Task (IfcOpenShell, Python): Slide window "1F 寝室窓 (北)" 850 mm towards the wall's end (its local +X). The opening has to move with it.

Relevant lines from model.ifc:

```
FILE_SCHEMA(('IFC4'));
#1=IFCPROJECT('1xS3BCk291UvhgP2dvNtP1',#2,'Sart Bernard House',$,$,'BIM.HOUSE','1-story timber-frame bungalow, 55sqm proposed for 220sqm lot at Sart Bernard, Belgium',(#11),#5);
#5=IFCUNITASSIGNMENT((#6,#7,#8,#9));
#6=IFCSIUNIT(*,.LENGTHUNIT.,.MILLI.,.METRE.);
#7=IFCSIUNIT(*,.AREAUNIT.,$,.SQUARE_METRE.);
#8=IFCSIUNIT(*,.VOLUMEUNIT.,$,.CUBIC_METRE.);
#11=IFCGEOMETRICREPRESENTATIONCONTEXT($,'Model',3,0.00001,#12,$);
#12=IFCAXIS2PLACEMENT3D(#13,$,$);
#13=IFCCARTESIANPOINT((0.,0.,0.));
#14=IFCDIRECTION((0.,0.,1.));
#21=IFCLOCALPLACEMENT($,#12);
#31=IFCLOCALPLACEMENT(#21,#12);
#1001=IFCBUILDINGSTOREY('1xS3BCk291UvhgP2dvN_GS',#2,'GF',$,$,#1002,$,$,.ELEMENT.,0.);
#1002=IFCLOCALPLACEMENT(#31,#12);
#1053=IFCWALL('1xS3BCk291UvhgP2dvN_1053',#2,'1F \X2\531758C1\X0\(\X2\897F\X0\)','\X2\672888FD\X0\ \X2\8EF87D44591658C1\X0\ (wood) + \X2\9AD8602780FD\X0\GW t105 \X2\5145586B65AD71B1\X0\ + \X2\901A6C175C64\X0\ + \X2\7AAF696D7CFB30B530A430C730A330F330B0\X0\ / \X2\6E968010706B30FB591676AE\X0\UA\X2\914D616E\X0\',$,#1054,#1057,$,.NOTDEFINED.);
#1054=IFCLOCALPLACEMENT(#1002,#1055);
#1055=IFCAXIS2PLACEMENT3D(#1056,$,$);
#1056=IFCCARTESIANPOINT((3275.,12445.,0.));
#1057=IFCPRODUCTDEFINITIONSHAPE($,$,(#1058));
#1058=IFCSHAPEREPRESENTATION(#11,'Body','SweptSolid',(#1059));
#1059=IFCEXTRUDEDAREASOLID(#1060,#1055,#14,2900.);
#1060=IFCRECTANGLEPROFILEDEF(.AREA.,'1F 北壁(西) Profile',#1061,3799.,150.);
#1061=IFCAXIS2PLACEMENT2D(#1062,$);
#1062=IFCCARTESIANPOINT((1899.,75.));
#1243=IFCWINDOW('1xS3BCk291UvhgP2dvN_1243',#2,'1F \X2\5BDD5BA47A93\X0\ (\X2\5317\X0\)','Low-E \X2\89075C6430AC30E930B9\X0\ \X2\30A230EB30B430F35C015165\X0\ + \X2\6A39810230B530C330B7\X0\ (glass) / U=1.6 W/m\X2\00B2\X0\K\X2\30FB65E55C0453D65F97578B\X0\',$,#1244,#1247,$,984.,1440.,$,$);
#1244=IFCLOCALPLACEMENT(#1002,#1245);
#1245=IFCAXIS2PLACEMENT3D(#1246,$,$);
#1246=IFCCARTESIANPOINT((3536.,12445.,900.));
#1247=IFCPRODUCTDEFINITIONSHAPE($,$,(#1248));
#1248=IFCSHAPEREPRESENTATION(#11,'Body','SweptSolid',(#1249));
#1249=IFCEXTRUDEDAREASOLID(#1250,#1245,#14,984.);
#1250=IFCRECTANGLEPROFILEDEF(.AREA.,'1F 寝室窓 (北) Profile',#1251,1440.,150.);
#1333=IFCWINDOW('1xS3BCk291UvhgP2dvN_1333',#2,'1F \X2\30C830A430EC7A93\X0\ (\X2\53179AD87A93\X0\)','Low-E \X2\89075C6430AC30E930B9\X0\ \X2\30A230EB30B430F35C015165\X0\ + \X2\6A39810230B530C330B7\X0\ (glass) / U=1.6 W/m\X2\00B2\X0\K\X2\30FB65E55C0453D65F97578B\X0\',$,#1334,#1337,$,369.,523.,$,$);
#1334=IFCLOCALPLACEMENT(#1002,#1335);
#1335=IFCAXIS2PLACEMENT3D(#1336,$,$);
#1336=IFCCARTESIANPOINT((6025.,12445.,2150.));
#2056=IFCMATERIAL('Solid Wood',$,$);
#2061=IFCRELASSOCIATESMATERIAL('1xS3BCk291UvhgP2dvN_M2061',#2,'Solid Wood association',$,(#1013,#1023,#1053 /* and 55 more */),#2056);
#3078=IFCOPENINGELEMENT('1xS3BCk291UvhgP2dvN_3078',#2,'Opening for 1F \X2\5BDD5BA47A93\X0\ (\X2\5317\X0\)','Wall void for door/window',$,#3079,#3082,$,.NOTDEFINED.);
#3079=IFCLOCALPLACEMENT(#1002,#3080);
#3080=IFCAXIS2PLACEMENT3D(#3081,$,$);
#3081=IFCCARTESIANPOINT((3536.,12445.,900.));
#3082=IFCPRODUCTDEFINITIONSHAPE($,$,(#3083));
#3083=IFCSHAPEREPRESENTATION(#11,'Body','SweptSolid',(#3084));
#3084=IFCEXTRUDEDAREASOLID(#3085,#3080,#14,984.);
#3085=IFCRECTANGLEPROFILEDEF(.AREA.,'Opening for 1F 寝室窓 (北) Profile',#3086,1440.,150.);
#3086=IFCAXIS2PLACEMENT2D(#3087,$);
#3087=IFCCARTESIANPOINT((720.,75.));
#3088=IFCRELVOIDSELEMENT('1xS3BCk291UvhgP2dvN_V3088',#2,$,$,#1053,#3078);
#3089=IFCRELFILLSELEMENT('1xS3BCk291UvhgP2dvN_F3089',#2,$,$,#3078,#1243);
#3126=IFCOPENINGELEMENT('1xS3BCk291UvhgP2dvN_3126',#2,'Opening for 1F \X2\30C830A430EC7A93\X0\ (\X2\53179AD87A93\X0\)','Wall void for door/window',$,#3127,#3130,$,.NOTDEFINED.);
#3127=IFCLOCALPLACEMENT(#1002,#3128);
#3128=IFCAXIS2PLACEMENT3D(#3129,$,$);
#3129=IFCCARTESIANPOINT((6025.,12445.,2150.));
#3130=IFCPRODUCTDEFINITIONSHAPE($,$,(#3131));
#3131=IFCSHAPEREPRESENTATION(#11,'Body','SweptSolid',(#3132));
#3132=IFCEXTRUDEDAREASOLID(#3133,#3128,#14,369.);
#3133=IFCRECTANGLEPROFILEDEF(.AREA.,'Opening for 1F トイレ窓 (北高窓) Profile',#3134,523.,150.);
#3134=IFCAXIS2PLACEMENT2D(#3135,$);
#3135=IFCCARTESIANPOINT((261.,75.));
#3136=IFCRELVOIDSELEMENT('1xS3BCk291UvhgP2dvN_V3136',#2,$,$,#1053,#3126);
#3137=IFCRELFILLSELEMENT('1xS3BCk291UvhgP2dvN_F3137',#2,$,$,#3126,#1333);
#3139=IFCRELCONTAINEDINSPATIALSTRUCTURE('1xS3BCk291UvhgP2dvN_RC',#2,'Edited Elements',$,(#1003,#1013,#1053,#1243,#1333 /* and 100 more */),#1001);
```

```python
import ifcopenshell
import ifcopenshell.api.geometry
import ifcopenshell.util.placement

model = ifcopenshell.open("model.ifc")

window = model.by_guid("1xS3BCk291UvhgP2dvN_1243")
opening = window.FillsVoids[0].RelatingOpeningElement
wall = opening.VoidsElements[0].RelatingBuildingElement

wall_matrix = ifcopenshell.util.placement.get_local_placement(wall.ObjectPlacement)
shift = wall_matrix[:3, 0] * 850.0
before = ifcopenshell.util.placement.get_local_placement(window.ObjectPlacement)[:3, 3].copy()

# The window is not placed relative to its opening, so move both.
for product in (opening, window):
    matrix = ifcopenshell.util.placement.get_local_placement(product.ObjectPlacement)
    matrix[:3, 3] += shift
    ifcopenshell.api.geometry.edit_object_placement(model, product=product, matrix=matrix, is_si=False)

after = ifcopenshell.util.placement.get_local_placement(window.ObjectPlacement)[:3, 3]
print("window moved by", (after - before).round(3) + 0.0)

model.write("model_rev.ifc")
```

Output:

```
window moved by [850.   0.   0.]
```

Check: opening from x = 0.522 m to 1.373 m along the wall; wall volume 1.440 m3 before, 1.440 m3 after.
